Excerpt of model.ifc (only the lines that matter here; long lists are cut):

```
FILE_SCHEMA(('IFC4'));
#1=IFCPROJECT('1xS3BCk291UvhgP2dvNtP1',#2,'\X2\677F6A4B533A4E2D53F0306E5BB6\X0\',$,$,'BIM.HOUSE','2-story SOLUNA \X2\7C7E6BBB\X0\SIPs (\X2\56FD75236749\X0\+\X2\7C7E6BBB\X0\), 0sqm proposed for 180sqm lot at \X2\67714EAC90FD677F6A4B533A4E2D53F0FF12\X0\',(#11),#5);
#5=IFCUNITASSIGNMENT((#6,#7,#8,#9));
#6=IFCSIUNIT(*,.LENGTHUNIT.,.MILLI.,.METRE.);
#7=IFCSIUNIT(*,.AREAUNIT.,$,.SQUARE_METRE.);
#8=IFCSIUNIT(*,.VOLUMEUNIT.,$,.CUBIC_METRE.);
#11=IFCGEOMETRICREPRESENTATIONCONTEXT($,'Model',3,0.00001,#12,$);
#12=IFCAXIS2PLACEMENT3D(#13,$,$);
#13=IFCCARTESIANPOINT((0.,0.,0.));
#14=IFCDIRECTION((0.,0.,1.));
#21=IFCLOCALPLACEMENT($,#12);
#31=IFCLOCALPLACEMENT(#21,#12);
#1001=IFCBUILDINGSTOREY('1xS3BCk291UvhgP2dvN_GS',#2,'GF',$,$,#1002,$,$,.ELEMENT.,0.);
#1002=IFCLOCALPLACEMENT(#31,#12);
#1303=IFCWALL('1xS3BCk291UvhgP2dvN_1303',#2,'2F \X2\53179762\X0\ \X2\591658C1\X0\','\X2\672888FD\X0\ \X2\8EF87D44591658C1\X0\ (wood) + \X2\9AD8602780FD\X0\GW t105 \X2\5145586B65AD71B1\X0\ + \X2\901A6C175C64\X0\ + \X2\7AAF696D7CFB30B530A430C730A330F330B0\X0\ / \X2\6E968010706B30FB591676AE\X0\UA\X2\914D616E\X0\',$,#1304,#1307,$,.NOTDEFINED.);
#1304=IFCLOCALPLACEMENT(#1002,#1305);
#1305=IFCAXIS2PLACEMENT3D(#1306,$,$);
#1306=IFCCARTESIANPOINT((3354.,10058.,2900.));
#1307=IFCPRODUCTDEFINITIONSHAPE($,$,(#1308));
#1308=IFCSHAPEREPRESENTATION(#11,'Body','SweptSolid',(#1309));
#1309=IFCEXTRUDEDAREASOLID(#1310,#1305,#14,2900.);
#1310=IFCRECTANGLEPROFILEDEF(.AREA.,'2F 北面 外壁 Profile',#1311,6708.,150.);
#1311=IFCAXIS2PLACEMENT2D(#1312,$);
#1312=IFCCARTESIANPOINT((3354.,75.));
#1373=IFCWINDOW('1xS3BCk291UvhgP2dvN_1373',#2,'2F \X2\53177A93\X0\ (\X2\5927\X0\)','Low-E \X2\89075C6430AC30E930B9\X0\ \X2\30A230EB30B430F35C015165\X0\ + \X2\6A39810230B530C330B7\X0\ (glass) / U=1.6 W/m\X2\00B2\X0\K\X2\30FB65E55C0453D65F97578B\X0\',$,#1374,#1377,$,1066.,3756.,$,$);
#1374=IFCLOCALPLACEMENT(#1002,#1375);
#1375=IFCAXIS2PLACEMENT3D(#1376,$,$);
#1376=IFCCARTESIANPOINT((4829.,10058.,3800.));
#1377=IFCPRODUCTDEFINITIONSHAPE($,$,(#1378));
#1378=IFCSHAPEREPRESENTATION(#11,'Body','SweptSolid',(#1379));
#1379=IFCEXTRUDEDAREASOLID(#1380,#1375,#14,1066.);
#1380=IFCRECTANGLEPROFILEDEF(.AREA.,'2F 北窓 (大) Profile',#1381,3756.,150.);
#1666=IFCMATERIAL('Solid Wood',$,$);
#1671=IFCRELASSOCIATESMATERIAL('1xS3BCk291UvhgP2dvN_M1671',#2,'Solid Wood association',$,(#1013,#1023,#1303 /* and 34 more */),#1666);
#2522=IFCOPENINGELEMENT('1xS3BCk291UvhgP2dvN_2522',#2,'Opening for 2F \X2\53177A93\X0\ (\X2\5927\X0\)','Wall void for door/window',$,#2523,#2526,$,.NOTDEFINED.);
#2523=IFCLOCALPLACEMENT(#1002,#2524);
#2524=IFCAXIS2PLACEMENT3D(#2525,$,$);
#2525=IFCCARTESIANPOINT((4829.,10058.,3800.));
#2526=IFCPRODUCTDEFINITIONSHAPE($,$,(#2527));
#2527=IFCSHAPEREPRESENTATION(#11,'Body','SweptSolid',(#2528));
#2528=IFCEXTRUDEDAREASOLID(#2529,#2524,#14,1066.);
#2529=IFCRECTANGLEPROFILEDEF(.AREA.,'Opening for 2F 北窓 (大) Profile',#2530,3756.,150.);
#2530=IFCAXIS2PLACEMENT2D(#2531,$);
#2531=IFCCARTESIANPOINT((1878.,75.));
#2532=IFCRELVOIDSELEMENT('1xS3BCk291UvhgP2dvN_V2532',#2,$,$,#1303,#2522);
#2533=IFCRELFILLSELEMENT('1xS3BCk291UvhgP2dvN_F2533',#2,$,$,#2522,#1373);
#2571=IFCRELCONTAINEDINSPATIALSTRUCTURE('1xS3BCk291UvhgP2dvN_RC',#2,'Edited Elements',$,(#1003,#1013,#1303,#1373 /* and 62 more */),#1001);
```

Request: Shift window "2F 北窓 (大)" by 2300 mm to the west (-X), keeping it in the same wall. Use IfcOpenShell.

```python
import ifcopenshell
import ifcopenshell.api.geometry
import ifcopenshell.util.placement
import ifcopenshell.util.unit

model = ifcopenshell.open("model.ifc")
unit_scale = ifcopenshell.util.unit.calculate_unit_scale(model)

window = model.by_guid("1xS3BCk291UvhgP2dvN_1373")
opening = window.FillsVoids[0].RelatingOpeningElement
wall = opening.VoidsElements[0].RelatingBuildingElement

wall_matrix = ifcopenshell.util.placement.get_local_placement(wall.ObjectPlacement)
shift = wall_matrix[:3, 0] * -2.3 / unit_scale
before = ifcopenshell.util.placement.get_local_placement(window.ObjectPlacement)[:3, 3].copy()

# The window is not placed relative to its opening, so move both.
for product in (opening, window):
    matrix = ifcopenshell.util.placement.get_local_placement(product.ObjectPlacement)
    matrix[:3, 3] += shift
    ifcopenshell.api.geometry.edit_object_placement(model, product=product, matrix=matrix, is_si=False)

after = ifcopenshell.util.placement.get_local_placement(window.ObjectPlacement)[:3, 3]
print("window moved by", (after - before).round(3) + 0.0)

model.write("model_updated.ifc")
```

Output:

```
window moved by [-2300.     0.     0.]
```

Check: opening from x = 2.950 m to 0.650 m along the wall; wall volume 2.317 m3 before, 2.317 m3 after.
